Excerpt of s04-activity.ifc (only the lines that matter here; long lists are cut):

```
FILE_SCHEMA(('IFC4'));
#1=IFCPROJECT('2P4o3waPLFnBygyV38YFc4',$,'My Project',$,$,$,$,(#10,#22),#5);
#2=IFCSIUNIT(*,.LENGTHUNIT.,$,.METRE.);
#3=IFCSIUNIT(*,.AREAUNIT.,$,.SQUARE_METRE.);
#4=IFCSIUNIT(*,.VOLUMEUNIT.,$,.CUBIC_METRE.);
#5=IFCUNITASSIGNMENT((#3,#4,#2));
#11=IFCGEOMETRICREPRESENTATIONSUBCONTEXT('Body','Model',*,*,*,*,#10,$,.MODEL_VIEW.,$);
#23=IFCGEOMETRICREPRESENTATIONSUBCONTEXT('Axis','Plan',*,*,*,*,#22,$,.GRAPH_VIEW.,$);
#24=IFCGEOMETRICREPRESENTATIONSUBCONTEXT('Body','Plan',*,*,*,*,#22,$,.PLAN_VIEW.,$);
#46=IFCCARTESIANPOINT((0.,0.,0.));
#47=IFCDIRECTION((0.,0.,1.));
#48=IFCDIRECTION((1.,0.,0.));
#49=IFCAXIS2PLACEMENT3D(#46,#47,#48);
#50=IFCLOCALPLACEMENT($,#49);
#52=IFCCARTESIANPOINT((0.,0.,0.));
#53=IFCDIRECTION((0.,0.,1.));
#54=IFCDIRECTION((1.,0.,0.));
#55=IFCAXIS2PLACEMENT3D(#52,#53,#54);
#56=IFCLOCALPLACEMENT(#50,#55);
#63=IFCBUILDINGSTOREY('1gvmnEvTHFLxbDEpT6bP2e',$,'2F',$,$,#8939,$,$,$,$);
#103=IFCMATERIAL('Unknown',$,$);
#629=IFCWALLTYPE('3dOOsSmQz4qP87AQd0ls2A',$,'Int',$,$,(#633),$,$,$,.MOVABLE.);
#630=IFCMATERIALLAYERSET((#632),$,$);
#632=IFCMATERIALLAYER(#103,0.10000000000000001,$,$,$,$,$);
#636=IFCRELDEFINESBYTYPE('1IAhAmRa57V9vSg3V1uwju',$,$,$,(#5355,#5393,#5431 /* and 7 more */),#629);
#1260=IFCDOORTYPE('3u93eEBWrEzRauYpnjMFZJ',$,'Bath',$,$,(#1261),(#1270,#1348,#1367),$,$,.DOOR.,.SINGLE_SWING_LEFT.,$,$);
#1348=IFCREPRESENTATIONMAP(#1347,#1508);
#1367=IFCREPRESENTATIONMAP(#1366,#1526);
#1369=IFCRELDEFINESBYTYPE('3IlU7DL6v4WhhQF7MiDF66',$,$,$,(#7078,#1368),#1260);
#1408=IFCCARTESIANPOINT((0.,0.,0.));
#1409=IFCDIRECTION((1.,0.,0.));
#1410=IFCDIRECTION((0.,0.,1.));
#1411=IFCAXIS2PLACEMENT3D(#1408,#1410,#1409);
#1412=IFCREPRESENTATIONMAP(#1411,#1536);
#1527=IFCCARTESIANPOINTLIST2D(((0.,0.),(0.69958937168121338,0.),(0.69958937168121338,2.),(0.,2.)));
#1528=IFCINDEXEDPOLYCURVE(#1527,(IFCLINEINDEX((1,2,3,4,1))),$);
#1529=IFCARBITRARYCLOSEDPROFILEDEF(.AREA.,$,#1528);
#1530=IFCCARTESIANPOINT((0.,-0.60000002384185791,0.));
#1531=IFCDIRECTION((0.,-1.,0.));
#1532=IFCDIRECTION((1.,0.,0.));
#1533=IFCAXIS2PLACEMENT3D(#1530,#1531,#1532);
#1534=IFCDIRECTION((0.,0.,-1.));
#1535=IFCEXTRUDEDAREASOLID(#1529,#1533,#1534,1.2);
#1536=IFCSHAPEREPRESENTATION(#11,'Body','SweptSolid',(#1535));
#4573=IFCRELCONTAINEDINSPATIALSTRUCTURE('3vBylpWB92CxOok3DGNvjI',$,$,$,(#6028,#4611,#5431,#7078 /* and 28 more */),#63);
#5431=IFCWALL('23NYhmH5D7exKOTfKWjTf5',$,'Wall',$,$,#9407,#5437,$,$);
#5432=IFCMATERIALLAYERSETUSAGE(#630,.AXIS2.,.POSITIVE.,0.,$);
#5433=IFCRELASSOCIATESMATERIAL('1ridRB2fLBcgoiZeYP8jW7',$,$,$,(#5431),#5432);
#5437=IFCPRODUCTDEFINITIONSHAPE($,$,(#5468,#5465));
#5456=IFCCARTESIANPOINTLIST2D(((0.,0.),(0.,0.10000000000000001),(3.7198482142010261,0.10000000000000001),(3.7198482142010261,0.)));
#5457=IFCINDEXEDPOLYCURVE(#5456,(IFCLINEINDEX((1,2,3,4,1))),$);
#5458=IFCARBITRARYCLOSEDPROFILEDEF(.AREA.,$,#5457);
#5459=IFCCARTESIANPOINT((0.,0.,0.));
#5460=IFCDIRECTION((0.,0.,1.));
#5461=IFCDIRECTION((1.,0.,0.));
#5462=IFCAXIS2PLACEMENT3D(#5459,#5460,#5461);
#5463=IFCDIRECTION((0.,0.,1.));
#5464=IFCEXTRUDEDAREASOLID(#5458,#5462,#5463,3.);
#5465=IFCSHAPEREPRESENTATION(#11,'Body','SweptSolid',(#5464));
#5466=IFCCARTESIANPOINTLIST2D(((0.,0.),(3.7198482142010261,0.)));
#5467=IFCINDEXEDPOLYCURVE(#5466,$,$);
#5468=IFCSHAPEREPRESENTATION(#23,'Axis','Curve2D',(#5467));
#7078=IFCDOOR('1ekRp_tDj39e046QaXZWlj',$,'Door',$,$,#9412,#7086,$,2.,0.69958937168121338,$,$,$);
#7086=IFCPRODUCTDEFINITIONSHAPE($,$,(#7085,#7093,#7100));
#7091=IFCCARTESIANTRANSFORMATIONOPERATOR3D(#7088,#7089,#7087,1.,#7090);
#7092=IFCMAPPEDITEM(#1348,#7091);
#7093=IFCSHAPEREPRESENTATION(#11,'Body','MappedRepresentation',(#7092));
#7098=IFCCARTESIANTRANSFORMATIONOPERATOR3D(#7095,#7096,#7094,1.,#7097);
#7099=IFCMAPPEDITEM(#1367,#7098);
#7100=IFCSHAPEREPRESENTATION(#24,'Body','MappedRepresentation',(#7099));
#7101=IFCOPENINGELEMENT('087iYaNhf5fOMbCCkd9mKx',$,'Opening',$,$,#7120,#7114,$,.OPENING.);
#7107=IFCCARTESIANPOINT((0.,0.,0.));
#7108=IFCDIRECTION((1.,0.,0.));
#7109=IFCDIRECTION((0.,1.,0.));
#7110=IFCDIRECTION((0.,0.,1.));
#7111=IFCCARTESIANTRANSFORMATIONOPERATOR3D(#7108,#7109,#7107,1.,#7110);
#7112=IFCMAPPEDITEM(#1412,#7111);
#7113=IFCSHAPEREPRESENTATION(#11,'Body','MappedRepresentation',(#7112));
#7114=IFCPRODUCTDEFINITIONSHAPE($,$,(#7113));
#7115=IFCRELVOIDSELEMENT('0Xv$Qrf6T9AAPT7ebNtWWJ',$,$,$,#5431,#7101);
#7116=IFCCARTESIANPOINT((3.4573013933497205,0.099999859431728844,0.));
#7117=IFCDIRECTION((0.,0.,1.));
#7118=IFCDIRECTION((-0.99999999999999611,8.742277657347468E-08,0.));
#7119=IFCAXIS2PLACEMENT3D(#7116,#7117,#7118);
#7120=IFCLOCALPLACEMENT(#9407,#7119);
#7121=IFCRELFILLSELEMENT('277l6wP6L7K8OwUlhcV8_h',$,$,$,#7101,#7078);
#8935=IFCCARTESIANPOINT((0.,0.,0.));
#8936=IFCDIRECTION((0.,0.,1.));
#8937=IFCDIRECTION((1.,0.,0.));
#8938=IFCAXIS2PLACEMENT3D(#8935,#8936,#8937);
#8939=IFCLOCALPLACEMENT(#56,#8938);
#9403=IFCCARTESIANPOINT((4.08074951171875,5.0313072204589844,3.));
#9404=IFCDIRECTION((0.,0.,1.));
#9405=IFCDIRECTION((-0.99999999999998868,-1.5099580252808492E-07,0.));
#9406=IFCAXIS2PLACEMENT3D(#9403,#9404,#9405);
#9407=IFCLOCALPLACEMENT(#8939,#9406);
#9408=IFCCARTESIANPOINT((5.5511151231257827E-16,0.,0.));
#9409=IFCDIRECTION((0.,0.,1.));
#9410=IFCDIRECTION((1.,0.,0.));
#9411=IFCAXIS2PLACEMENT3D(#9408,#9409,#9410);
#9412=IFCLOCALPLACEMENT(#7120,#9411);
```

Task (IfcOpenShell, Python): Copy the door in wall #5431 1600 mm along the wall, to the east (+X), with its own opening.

```python
import ifcopenshell
import ifcopenshell.api.feature
import ifcopenshell.api.geometry
import ifcopenshell.api.root
import ifcopenshell.geom
import ifcopenshell.util.element
import ifcopenshell.util.placement
import ifcopenshell.util.shape
import ifcopenshell.util.unit

model = ifcopenshell.open("s04-activity.ifc")
unit_scale = ifcopenshell.util.unit.calculate_unit_scale(model)
settings = ifcopenshell.geom.settings()


def volume(element):
    """Net volume in cubic metres, openings subtracted."""
    shape = ifcopenshell.geom.create_shape(settings, element)
    return ifcopenshell.util.shape.get_volume(shape.geometry)


door = model.by_id(7078)
opening = door.FillsVoids[0].RelatingOpeningElement
wall = opening.VoidsElements[0].RelatingBuildingElement
before = volume(wall)
shift = ifcopenshell.util.placement.get_local_placement(wall.ObjectPlacement)[:3, 0] * -1.6 / unit_scale

# copy_class copies the void relationship, type, container and properties, but no geometry.
new_opening = ifcopenshell.api.root.copy_class(model, product=opening)
new_opening.Representation = ifcopenshell.util.element.copy_deep(
    model, opening.Representation, exclude=["IfcGeometricRepresentationContext", "IfcRepresentationMap"]
)
new_door = ifcopenshell.api.root.copy_class(model, product=door)
new_door.Representation = ifcopenshell.util.element.copy_deep(
    model, door.Representation, exclude=["IfcGeometricRepresentationContext", "IfcRepresentationMap"]
)
ifcopenshell.api.feature.add_filling(model, opening=new_opening, element=new_door)

for old, new in ((opening, new_opening), (door, new_door)):
    matrix = ifcopenshell.util.placement.get_local_placement(old.ObjectPlacement)
    matrix[:3, 3] += shift
    ifcopenshell.api.geometry.edit_object_placement(model, product=new, matrix=matrix, is_si=False)

after = volume(wall)

print(f"wall volume {before:.3f} -> {after:.3f} m3")

model.write("s04-activity-out.ifc")
```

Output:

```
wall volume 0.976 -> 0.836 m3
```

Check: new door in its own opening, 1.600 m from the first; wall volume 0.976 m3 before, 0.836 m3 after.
